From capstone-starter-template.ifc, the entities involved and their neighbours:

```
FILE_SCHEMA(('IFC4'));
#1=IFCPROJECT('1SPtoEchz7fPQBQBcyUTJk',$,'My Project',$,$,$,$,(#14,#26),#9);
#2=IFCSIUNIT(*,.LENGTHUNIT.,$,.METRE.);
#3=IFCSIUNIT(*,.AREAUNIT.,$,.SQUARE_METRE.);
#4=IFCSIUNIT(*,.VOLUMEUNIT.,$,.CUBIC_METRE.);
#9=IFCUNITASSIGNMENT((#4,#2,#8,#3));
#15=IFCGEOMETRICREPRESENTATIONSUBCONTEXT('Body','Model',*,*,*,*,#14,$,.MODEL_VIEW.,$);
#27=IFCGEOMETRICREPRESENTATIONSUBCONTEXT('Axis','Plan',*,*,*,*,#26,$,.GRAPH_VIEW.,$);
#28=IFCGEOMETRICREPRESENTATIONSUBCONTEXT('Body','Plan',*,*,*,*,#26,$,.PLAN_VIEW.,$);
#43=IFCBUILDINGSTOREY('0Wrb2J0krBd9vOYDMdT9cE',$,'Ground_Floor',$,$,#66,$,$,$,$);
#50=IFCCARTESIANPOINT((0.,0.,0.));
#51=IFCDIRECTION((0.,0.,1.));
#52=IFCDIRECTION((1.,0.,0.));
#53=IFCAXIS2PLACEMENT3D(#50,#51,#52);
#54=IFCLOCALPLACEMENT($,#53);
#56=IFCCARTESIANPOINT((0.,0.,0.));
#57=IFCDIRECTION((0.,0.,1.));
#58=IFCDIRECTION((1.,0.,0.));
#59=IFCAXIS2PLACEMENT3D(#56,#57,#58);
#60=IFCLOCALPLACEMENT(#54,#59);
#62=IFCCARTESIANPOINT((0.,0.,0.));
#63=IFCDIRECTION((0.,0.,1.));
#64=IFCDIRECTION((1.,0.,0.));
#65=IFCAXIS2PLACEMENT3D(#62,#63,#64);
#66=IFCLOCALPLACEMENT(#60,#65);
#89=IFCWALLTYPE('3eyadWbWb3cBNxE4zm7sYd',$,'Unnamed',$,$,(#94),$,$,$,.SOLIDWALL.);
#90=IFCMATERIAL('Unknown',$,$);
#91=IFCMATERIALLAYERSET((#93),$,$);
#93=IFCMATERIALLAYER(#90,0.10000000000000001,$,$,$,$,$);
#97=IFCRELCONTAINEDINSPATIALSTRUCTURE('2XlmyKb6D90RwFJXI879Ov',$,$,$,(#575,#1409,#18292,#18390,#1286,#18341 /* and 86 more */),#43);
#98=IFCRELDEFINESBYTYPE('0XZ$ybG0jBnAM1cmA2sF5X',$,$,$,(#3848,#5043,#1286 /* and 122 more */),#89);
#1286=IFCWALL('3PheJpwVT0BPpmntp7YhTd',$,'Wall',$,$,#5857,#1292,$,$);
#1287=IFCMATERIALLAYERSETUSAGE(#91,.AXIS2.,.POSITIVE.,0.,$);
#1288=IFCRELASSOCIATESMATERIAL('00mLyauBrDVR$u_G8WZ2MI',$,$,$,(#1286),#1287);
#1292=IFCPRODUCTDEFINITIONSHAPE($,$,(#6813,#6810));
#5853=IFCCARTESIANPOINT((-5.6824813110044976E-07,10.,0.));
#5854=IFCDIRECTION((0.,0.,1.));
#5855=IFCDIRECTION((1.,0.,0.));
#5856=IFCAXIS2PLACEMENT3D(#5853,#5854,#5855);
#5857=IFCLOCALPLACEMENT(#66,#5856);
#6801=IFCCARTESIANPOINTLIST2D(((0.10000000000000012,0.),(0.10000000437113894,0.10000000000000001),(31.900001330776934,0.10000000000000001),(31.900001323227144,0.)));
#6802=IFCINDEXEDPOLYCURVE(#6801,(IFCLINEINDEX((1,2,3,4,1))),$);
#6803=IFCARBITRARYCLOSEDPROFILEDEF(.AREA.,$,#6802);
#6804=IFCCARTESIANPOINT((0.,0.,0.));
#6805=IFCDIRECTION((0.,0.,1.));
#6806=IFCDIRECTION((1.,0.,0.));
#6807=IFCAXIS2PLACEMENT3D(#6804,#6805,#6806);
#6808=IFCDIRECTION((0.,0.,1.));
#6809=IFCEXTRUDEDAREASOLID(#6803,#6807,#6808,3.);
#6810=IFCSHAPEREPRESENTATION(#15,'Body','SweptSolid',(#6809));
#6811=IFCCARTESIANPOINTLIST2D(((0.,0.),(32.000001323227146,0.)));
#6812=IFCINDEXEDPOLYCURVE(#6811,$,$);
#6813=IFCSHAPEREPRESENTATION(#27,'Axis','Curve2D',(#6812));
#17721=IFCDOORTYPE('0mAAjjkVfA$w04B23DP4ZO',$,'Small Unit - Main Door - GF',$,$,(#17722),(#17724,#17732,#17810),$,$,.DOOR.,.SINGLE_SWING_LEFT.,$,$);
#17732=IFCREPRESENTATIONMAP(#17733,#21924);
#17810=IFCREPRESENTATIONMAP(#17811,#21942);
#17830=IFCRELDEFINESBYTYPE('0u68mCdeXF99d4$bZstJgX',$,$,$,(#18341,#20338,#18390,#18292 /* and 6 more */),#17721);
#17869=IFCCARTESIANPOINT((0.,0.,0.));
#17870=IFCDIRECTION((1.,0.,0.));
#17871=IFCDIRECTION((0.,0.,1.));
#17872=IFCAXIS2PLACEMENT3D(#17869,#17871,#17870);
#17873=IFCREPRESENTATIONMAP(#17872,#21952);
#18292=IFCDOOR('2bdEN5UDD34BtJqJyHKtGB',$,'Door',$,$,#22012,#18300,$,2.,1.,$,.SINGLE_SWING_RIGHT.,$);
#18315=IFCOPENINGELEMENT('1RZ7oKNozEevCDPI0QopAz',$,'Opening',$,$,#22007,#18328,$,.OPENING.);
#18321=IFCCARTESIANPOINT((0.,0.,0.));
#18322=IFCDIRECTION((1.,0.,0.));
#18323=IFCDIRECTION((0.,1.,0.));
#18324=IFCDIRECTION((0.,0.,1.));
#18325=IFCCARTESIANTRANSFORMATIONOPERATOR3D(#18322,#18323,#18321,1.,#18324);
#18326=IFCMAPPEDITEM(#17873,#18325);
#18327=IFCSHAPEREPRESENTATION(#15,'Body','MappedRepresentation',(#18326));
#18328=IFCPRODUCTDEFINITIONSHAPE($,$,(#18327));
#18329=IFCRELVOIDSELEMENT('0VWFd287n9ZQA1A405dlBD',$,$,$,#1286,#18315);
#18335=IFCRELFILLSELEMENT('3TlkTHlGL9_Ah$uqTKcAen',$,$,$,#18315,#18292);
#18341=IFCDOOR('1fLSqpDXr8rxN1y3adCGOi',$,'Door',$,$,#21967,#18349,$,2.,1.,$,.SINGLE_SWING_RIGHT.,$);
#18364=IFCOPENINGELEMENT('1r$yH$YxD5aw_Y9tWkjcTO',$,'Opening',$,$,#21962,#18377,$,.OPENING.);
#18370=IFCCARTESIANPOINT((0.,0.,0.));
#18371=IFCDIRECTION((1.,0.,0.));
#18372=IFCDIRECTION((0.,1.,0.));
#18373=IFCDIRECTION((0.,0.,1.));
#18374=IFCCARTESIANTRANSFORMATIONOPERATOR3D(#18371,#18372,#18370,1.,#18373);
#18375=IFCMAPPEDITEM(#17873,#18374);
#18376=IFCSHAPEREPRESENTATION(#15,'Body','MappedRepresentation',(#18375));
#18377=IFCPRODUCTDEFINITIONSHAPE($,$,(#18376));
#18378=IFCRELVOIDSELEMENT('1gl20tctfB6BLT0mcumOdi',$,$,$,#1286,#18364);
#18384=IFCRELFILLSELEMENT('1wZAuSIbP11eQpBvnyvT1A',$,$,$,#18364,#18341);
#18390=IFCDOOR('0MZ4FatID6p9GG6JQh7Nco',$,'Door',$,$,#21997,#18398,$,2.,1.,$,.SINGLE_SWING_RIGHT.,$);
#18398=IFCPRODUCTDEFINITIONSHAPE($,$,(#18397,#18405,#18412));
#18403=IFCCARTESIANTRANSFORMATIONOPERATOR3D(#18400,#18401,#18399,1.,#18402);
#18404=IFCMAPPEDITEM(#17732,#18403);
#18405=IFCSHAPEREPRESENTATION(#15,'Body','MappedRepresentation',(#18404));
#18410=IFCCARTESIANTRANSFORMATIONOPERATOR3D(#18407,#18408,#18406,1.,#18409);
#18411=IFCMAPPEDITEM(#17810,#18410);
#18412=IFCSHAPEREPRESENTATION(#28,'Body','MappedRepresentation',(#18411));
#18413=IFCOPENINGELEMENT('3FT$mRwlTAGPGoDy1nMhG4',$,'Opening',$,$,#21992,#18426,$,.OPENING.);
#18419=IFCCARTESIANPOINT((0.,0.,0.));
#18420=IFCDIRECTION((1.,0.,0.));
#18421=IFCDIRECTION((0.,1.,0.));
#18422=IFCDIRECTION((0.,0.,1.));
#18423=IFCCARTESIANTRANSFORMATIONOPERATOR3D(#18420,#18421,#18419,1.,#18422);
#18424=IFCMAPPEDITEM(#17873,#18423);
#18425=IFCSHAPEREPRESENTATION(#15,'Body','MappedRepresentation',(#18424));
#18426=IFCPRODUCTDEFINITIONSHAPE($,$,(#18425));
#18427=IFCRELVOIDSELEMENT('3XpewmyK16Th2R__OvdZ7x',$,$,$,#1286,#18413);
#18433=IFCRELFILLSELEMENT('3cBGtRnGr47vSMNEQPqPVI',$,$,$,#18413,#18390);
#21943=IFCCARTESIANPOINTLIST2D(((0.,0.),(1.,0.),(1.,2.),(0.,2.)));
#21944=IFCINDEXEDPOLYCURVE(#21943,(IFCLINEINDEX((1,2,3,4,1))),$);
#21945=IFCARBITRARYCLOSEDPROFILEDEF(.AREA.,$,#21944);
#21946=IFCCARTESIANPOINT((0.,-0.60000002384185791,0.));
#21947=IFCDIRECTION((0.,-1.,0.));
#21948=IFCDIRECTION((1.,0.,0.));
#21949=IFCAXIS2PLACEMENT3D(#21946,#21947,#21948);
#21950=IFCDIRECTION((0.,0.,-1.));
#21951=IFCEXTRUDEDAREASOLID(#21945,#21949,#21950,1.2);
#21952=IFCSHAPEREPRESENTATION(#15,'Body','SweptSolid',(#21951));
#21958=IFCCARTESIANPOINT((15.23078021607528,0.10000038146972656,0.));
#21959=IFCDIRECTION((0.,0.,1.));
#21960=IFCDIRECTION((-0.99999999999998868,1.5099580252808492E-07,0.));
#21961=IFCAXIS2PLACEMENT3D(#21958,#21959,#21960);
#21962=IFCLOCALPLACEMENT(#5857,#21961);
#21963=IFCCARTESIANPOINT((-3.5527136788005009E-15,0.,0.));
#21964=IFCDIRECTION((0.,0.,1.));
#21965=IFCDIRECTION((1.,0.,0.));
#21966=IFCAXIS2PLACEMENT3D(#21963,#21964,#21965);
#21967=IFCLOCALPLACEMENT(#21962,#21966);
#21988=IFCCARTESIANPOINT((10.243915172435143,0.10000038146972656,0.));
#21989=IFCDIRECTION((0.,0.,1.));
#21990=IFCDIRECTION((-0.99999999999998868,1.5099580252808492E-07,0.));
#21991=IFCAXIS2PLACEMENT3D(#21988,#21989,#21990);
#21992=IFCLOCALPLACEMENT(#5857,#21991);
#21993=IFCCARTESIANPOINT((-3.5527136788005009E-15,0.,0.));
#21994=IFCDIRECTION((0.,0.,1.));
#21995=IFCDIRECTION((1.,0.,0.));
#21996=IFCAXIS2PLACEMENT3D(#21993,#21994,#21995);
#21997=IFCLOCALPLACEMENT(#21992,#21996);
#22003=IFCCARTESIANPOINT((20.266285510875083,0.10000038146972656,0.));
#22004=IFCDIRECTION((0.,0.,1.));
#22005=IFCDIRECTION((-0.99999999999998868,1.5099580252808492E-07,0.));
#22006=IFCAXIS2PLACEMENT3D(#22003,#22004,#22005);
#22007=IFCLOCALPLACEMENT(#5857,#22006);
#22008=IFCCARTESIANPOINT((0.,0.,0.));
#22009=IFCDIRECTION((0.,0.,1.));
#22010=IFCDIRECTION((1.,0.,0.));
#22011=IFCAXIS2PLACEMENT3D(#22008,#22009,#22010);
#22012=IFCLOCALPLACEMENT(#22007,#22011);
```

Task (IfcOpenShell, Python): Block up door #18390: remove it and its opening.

```python
import ifcopenshell
import ifcopenshell.api.feature
import ifcopenshell.api.root
import ifcopenshell.geom
import ifcopenshell.util.shape

model = ifcopenshell.open("capstone-starter-template.ifc")
settings = ifcopenshell.geom.settings()


def volume(element):
    """Net volume in cubic metres, openings subtracted."""
    shape = ifcopenshell.geom.create_shape(settings, element)
    return ifcopenshell.util.shape.get_volume(shape.geometry)


door = model.by_guid("0MZ4FatID6p9GG6JQh7Nco")
opening = door.FillsVoids[0].RelatingOpeningElement
wall = opening.VoidsElements[0].RelatingBuildingElement
before = volume(wall)

ifcopenshell.api.root.remove_product(model, product=door)
ifcopenshell.api.feature.remove_feature(model, feature=opening)

after = volume(wall)

print(f"wall volume {before:.3f} -> {after:.3f} m3")

model.write("capstone-starter-template_updated.ifc")
```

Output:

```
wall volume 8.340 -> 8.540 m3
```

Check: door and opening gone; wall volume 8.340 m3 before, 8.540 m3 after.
